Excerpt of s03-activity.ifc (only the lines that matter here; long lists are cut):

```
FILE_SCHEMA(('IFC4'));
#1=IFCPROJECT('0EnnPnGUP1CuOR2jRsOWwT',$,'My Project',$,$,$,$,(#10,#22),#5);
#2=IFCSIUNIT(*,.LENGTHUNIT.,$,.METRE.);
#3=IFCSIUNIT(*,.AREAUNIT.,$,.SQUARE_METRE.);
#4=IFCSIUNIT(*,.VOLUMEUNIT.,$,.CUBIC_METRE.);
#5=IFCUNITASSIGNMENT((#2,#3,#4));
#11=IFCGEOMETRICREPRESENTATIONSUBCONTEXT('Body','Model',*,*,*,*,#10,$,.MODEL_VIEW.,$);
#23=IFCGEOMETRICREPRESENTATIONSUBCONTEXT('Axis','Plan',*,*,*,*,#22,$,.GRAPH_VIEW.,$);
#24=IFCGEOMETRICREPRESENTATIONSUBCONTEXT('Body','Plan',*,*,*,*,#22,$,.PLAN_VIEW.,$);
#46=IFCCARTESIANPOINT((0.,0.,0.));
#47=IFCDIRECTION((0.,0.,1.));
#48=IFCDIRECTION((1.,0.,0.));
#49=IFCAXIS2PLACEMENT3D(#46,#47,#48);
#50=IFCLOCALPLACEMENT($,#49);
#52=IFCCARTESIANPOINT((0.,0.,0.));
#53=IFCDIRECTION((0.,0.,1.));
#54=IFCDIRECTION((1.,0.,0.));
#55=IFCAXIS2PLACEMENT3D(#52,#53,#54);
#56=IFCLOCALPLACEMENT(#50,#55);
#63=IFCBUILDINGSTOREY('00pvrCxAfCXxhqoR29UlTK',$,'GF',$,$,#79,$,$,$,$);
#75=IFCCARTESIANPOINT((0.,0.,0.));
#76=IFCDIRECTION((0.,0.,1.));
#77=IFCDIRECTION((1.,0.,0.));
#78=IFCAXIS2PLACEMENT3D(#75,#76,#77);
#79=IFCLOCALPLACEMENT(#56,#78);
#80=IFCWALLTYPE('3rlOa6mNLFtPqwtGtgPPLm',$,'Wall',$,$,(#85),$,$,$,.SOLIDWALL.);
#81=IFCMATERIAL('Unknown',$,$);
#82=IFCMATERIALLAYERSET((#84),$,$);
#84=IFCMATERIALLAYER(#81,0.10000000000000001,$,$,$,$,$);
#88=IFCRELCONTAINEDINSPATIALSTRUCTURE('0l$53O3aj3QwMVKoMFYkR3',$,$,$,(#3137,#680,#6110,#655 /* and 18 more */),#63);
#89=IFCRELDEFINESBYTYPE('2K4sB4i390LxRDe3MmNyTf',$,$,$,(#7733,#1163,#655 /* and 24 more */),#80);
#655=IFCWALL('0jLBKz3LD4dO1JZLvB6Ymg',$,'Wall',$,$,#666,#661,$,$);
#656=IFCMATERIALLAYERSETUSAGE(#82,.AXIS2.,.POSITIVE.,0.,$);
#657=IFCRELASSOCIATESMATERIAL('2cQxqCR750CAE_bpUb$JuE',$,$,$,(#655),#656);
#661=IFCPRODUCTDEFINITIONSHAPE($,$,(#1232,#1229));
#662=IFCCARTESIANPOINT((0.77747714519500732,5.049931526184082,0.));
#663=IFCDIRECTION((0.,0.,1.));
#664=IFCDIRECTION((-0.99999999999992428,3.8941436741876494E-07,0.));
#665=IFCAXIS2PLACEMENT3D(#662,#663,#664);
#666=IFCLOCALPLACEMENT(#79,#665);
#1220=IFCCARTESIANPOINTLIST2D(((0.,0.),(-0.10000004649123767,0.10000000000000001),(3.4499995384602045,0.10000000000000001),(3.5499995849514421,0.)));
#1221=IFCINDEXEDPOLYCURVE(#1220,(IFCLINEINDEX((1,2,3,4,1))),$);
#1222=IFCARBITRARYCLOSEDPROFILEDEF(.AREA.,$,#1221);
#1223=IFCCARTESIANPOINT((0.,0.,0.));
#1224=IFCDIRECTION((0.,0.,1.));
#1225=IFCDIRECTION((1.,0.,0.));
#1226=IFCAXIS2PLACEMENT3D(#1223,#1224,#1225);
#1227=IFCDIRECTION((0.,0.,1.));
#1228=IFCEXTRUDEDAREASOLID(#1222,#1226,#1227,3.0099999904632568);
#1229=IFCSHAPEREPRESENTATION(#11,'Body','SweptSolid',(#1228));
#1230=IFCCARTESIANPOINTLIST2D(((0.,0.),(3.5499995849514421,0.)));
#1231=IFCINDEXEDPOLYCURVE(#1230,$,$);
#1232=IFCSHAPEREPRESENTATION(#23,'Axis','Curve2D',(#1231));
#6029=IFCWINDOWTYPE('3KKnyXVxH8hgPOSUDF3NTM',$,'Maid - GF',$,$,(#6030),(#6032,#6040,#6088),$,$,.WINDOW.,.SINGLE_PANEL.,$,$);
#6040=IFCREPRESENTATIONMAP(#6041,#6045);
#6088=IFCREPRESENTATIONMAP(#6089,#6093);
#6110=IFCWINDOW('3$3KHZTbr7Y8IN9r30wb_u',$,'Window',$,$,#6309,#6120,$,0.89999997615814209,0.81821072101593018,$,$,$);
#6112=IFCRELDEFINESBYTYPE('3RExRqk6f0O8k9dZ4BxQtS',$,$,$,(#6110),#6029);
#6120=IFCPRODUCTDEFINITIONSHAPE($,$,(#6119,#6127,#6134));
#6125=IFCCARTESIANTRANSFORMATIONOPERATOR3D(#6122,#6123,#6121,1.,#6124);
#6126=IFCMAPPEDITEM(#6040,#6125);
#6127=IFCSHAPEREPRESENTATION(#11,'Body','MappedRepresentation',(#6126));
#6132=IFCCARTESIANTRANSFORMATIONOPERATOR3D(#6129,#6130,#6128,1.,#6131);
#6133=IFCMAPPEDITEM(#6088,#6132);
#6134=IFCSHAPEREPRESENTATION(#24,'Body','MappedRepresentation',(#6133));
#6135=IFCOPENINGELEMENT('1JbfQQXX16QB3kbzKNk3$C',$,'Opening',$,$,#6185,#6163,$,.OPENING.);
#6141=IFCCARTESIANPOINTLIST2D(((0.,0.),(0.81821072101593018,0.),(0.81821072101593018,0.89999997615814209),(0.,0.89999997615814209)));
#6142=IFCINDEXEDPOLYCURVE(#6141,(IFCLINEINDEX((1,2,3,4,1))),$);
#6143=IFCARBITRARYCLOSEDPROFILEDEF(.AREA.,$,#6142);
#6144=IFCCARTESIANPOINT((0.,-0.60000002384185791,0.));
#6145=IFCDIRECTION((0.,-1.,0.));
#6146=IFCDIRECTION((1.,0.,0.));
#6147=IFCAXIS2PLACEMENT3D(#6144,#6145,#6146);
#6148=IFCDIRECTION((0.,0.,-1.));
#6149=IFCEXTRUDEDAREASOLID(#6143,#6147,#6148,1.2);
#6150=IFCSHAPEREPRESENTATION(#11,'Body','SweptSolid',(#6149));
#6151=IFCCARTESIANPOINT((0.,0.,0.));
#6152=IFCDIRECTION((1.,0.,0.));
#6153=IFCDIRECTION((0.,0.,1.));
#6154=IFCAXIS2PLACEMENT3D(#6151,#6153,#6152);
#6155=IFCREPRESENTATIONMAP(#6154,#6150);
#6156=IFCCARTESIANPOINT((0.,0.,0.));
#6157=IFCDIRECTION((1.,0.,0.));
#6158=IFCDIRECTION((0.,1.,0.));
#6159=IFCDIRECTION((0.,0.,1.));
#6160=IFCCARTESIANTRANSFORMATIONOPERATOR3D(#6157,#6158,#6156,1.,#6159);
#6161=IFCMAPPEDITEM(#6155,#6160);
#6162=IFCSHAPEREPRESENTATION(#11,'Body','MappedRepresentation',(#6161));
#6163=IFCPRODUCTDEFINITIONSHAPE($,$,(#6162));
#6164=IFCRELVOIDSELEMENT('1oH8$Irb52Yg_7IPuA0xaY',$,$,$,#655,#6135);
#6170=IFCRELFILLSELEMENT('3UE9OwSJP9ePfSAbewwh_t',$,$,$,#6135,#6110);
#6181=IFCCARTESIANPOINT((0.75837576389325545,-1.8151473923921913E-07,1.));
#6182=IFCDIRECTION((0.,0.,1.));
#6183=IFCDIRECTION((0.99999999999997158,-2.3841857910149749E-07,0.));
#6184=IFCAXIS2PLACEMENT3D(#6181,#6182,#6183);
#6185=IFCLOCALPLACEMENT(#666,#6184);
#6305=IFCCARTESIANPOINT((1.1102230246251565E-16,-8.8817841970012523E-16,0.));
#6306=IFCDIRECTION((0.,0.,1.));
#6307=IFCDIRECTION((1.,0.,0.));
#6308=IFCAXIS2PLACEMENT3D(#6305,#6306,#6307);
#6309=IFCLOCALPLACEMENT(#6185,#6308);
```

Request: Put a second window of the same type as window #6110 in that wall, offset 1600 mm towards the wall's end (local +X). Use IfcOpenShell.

```python
import ifcopenshell
import ifcopenshell.api.feature
import ifcopenshell.api.geometry
import ifcopenshell.api.root
import ifcopenshell.geom
import ifcopenshell.util.element
import ifcopenshell.util.placement
import ifcopenshell.util.shape
import ifcopenshell.util.unit

model = ifcopenshell.open("s03-activity.ifc")
unit_scale = ifcopenshell.util.unit.calculate_unit_scale(model)
settings = ifcopenshell.geom.settings()


def volume(element):
    """Net volume in cubic metres, openings subtracted."""
    shape = ifcopenshell.geom.create_shape(settings, element)
    return ifcopenshell.util.shape.get_volume(shape.geometry)


window = model.by_id(6110)
opening = window.FillsVoids[0].RelatingOpeningElement
wall = opening.VoidsElements[0].RelatingBuildingElement
before = volume(wall)
shift = ifcopenshell.util.placement.get_local_placement(wall.ObjectPlacement)[:3, 0] * 1.6 / unit_scale

# copy_class copies the void relationship, type, container and properties, but no geometry.
new_opening = ifcopenshell.api.root.copy_class(model, product=opening)
new_opening.Representation = ifcopenshell.util.element.copy_deep(
    model, opening.Representation, exclude=["IfcGeometricRepresentationContext", "IfcRepresentationMap"]
)
new_window = ifcopenshell.api.root.copy_class(model, product=window)
new_window.Representation = ifcopenshell.util.element.copy_deep(
    model, window.Representation, exclude=["IfcGeometricRepresentationContext", "IfcRepresentationMap"]
)
ifcopenshell.api.feature.add_filling(model, opening=new_opening, element=new_window)

for old, new in ((opening, new_opening), (window, new_window)):
    matrix = ifcopenshell.util.placement.get_local_placement(old.ObjectPlacement)
    matrix[:3, 3] += shift
    ifcopenshell.api.geometry.edit_object_placement(model, product=new, matrix=matrix, is_si=False)

after = volume(wall)

print(f"wall volume {before:.3f} -> {after:.3f} m3")

model.write("s03-activity-out.ifc")
```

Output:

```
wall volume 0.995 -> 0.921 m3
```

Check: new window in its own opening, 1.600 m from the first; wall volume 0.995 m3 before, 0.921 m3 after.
